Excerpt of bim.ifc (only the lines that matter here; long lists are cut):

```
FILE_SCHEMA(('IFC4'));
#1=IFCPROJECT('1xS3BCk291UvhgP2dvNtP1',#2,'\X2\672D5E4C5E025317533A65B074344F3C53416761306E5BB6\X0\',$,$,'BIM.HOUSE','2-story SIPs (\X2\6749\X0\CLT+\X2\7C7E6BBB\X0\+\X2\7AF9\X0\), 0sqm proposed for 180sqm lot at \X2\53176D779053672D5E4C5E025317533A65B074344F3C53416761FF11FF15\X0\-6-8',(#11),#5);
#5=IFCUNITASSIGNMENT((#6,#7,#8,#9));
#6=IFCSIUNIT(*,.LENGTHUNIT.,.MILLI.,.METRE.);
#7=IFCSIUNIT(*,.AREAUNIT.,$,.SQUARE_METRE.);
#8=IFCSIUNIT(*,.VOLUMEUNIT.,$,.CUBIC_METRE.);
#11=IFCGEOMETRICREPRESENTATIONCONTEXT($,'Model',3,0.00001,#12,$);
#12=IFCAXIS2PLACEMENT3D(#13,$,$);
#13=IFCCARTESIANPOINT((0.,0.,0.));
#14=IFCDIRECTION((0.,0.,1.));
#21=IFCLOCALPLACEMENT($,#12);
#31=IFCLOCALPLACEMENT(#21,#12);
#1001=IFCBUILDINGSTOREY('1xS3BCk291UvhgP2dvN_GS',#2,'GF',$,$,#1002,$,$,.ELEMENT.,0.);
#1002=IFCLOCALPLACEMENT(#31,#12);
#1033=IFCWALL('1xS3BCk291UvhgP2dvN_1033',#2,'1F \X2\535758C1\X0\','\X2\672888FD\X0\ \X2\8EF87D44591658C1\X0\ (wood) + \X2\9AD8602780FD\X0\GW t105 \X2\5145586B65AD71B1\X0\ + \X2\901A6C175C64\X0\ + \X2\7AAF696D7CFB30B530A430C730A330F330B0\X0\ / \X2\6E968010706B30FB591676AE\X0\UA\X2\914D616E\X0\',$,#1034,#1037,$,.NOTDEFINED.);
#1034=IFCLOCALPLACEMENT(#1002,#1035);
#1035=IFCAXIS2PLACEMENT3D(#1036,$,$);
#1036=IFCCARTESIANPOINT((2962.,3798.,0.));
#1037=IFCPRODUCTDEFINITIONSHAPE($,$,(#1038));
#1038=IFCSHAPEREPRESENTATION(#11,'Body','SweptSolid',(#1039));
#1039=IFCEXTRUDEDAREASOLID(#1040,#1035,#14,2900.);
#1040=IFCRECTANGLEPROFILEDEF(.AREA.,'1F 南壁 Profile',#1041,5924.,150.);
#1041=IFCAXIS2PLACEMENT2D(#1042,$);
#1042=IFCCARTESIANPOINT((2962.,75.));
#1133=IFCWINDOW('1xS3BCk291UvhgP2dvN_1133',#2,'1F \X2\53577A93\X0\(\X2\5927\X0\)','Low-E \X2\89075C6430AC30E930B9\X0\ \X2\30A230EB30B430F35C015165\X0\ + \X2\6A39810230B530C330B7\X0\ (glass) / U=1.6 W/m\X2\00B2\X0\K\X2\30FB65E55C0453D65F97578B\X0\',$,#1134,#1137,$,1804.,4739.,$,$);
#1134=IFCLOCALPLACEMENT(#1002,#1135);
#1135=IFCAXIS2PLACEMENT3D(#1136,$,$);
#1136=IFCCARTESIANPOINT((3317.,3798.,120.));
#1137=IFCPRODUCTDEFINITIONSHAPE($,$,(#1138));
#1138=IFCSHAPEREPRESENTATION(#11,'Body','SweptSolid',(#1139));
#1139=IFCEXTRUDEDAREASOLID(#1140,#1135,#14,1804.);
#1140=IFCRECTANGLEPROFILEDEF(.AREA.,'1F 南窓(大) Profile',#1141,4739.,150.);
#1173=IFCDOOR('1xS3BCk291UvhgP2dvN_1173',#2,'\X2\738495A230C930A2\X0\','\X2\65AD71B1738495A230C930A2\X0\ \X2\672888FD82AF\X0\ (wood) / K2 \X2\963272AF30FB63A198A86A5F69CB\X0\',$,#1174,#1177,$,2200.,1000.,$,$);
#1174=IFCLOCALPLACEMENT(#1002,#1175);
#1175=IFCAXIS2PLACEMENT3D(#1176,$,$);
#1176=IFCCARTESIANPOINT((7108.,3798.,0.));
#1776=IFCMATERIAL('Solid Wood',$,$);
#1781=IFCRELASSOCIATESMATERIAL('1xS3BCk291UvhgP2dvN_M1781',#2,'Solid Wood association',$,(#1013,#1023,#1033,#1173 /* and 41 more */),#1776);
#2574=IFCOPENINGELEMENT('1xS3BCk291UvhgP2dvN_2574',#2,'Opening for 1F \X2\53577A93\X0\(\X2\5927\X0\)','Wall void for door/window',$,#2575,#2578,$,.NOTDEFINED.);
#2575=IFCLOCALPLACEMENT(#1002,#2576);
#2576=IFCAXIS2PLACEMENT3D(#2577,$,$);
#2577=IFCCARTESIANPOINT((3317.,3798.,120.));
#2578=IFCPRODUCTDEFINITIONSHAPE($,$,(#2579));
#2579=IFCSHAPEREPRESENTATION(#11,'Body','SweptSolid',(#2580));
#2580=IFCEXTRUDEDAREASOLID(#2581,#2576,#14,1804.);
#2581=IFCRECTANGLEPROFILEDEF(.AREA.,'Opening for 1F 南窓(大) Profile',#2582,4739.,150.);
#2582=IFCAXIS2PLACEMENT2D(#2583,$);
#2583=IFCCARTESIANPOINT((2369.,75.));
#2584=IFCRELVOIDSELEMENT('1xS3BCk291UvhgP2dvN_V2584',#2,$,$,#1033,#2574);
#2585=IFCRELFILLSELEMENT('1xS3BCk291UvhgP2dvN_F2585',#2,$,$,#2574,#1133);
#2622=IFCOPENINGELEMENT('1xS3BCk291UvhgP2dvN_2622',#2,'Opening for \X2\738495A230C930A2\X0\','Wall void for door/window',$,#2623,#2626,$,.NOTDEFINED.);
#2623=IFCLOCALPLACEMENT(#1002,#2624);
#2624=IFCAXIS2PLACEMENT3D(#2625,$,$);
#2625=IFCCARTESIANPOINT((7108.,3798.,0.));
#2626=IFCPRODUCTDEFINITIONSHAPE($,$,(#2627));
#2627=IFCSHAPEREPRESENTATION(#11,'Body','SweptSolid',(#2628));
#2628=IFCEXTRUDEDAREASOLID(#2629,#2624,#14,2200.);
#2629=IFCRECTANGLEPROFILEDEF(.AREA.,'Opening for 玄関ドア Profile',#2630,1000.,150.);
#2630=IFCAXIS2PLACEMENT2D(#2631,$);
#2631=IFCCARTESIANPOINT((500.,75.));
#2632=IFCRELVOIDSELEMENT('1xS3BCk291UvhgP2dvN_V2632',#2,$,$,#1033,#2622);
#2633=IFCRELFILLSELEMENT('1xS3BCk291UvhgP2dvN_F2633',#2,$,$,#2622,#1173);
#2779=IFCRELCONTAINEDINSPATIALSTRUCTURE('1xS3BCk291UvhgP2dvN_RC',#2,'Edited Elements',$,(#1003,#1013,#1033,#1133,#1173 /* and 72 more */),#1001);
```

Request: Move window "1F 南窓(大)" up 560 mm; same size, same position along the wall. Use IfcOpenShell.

```python
import numpy as np
import ifcopenshell
import ifcopenshell.api.geometry
import ifcopenshell.util.placement
import ifcopenshell.util.unit

model = ifcopenshell.open("bim.ifc")
unit_scale = ifcopenshell.util.unit.calculate_unit_scale(model)

window = model.by_guid("1xS3BCk291UvhgP2dvN_1133")
opening = window.FillsVoids[0].RelatingOpeningElement
dz = 0.56 / unit_scale

shift = np.array([0.0, 0.0, dz])
# The window is not placed relative to its opening, so move both.
for product in (opening, window):
    matrix = ifcopenshell.util.placement.get_local_placement(product.ObjectPlacement)
    matrix[:3, 3] += shift
    ifcopenshell.api.geometry.edit_object_placement(model, product=product, matrix=matrix, is_si=False)

print(f"moved by {dz * unit_scale:+.3f} m")

model.write("bim_v2.ifc")
```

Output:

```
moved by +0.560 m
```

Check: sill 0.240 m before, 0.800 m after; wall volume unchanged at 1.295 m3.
